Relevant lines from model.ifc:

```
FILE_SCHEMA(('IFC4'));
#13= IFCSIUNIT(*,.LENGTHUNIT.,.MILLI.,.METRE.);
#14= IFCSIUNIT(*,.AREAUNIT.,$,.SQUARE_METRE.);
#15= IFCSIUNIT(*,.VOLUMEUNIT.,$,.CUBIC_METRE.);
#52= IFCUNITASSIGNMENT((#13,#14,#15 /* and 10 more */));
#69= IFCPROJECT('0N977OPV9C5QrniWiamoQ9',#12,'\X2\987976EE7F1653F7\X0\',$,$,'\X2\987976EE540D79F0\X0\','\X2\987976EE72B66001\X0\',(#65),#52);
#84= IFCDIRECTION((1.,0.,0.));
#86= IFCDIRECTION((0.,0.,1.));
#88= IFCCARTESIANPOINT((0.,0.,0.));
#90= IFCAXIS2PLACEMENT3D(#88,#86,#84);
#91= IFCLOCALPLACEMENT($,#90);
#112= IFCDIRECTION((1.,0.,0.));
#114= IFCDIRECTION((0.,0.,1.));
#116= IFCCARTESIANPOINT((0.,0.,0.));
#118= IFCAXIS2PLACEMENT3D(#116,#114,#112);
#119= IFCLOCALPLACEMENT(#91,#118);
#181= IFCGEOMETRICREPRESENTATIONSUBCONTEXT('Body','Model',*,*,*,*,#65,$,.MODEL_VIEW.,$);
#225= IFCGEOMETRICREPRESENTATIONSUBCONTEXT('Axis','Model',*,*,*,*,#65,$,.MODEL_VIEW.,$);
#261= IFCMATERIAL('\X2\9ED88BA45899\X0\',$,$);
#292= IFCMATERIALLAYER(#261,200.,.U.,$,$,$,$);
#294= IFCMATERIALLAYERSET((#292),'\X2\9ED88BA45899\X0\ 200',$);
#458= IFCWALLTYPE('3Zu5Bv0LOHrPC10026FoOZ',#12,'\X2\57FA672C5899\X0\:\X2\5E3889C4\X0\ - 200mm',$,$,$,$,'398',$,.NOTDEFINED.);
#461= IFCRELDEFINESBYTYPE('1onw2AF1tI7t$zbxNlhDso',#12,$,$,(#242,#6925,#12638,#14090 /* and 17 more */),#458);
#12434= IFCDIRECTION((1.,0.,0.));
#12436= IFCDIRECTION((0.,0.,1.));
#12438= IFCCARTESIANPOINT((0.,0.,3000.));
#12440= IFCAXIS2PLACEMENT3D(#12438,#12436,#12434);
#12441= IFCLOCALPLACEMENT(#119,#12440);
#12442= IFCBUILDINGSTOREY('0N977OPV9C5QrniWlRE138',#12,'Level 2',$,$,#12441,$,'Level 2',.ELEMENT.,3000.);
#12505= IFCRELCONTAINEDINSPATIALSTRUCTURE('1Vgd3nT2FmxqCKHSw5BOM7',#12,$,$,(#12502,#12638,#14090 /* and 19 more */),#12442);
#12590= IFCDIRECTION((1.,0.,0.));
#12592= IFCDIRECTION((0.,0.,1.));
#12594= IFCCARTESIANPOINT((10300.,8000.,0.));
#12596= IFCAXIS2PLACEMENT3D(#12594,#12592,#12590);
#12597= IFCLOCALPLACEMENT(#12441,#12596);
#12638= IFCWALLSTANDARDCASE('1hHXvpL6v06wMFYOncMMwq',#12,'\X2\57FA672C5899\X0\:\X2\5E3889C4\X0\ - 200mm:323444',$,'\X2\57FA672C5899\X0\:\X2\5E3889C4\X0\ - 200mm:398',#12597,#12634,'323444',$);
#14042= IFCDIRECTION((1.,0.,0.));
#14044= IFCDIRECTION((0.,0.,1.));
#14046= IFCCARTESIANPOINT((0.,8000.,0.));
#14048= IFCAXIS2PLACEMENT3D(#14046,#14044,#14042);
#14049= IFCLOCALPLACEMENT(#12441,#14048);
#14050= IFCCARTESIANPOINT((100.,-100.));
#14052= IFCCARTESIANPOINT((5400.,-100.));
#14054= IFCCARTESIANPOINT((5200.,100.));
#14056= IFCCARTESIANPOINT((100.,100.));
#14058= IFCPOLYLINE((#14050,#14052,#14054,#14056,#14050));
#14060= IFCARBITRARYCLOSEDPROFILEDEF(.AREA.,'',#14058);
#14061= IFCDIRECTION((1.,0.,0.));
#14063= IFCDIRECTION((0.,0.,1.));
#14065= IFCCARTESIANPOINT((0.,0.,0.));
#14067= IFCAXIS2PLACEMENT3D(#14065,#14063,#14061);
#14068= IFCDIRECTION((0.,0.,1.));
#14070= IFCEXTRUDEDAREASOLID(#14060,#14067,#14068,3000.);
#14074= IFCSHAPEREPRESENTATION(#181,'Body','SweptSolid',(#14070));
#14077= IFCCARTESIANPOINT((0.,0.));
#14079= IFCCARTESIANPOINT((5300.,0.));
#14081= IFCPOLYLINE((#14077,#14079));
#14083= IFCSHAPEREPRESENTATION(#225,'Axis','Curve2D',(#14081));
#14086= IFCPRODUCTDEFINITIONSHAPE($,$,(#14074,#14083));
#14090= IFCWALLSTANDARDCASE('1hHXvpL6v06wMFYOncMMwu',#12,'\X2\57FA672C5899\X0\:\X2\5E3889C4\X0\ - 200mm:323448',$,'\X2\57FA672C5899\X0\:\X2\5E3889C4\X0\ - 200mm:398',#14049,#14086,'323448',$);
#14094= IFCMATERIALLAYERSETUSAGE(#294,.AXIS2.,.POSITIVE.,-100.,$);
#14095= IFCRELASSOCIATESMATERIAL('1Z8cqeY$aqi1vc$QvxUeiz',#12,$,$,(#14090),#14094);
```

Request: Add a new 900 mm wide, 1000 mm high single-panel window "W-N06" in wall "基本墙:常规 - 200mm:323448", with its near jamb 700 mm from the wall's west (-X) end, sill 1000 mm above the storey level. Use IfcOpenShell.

```python
import numpy as np
import ifcopenshell
import ifcopenshell.api.feature
import ifcopenshell.api.geometry
import ifcopenshell.api.root
import ifcopenshell.api.spatial
import ifcopenshell.geom
import ifcopenshell.util.element
import ifcopenshell.util.placement
import ifcopenshell.util.representation
import ifcopenshell.util.shape
import ifcopenshell.util.unit

model = ifcopenshell.open("model.ifc")
unit_scale = ifcopenshell.util.unit.calculate_unit_scale(model)
settings = ifcopenshell.geom.settings()


def volume(element):
    """Net volume in cubic metres, openings subtracted."""
    shape = ifcopenshell.geom.create_shape(settings, element)
    return ifcopenshell.util.shape.get_volume(shape.geometry)


wall = model.by_id(14090)
storey = ifcopenshell.util.element.get_container(wall, ifc_class="IfcBuildingStorey")
context = ifcopenshell.util.representation.get_context(model, "Model", "Body", "MODEL_VIEW")
before = volume(wall)

width, height, from_end, sill = 0.9, 1, 0.7, 1  # metres

# The wall runs along its own X axis, and the end named is its -X end.
wall_shape = ifcopenshell.geom.create_shape(settings, wall)
x, y, z = ifcopenshell.util.shape.get_vertices(wall_shape.geometry).T
start = x.min() + from_end
face, thickness = float(y.min()), float(y.max() - y.min())
wall_matrix = ifcopenshell.util.placement.get_local_placement(wall.ObjectPlacement)
level = ifcopenshell.util.placement.get_local_placement(storey.ObjectPlacement)[2, 3]


def in_wall(x, y):
    """Placement at x, y metres in the wall's axes, at sill height."""
    matrix = wall_matrix.copy()
    matrix[:, 3] = wall_matrix @ np.array([x / unit_scale, y / unit_scale, 0.0, 1.0])
    matrix[2, 3] = level + sill / unit_scale
    return matrix


# Opening: a box that overshoots both wall faces by 50 mm.
opening = ifcopenshell.api.root.create_entity(model, ifc_class="IfcOpeningElement", predefined_type="OPENING")
box = ifcopenshell.api.geometry.add_wall_representation(
    model, context=context, length=width, height=height, thickness=thickness + 0.1
)
ifcopenshell.api.geometry.assign_representation(model, product=opening, representation=box)
ifcopenshell.api.geometry.edit_object_placement(model, product=opening, matrix=in_wall(start, face - 0.05), is_si=False)
ifcopenshell.api.feature.add_feature(model, feature=opening, element=wall)

window = ifcopenshell.api.root.create_entity(model, ifc_class="IfcWindow", name="W-N06", predefined_type="WINDOW")
window.OverallWidth, window.OverallHeight = width / unit_scale, height / unit_scale
window.PartitioningType = "SINGLE_PANEL"
body = ifcopenshell.api.geometry.add_window_representation(
    model,
    context=context,
    overall_width=window.OverallWidth,
    overall_height=window.OverallHeight,
    partition_type="SINGLE_PANEL",
)
ifcopenshell.api.geometry.assign_representation(model, product=window, representation=body)
ifcopenshell.api.spatial.assign_container(model, products=[window], relating_structure=storey)
ifcopenshell.api.feature.add_filling(model, opening=opening, element=window)

# Centre the window in the wall's thickness.
ifcopenshell.api.geometry.edit_object_placement(model, product=window, matrix=in_wall(start, face), is_si=False)
window_shape = ifcopenshell.geom.create_shape(settings, window)
depth = ifcopenshell.util.shape.get_vertices(window_shape.geometry)[:, 1]
offset = face + thickness / 2 - (depth.min() + depth.max()) / 2
ifcopenshell.api.geometry.edit_object_placement(model, product=window, matrix=in_wall(start, offset), is_si=False)

after = volume(wall)

print(f"wall volume {before:.3f} -> {after:.3f} m3")

model.write("model_edited.ifc")
```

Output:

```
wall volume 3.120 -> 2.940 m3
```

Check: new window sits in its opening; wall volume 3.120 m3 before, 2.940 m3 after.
